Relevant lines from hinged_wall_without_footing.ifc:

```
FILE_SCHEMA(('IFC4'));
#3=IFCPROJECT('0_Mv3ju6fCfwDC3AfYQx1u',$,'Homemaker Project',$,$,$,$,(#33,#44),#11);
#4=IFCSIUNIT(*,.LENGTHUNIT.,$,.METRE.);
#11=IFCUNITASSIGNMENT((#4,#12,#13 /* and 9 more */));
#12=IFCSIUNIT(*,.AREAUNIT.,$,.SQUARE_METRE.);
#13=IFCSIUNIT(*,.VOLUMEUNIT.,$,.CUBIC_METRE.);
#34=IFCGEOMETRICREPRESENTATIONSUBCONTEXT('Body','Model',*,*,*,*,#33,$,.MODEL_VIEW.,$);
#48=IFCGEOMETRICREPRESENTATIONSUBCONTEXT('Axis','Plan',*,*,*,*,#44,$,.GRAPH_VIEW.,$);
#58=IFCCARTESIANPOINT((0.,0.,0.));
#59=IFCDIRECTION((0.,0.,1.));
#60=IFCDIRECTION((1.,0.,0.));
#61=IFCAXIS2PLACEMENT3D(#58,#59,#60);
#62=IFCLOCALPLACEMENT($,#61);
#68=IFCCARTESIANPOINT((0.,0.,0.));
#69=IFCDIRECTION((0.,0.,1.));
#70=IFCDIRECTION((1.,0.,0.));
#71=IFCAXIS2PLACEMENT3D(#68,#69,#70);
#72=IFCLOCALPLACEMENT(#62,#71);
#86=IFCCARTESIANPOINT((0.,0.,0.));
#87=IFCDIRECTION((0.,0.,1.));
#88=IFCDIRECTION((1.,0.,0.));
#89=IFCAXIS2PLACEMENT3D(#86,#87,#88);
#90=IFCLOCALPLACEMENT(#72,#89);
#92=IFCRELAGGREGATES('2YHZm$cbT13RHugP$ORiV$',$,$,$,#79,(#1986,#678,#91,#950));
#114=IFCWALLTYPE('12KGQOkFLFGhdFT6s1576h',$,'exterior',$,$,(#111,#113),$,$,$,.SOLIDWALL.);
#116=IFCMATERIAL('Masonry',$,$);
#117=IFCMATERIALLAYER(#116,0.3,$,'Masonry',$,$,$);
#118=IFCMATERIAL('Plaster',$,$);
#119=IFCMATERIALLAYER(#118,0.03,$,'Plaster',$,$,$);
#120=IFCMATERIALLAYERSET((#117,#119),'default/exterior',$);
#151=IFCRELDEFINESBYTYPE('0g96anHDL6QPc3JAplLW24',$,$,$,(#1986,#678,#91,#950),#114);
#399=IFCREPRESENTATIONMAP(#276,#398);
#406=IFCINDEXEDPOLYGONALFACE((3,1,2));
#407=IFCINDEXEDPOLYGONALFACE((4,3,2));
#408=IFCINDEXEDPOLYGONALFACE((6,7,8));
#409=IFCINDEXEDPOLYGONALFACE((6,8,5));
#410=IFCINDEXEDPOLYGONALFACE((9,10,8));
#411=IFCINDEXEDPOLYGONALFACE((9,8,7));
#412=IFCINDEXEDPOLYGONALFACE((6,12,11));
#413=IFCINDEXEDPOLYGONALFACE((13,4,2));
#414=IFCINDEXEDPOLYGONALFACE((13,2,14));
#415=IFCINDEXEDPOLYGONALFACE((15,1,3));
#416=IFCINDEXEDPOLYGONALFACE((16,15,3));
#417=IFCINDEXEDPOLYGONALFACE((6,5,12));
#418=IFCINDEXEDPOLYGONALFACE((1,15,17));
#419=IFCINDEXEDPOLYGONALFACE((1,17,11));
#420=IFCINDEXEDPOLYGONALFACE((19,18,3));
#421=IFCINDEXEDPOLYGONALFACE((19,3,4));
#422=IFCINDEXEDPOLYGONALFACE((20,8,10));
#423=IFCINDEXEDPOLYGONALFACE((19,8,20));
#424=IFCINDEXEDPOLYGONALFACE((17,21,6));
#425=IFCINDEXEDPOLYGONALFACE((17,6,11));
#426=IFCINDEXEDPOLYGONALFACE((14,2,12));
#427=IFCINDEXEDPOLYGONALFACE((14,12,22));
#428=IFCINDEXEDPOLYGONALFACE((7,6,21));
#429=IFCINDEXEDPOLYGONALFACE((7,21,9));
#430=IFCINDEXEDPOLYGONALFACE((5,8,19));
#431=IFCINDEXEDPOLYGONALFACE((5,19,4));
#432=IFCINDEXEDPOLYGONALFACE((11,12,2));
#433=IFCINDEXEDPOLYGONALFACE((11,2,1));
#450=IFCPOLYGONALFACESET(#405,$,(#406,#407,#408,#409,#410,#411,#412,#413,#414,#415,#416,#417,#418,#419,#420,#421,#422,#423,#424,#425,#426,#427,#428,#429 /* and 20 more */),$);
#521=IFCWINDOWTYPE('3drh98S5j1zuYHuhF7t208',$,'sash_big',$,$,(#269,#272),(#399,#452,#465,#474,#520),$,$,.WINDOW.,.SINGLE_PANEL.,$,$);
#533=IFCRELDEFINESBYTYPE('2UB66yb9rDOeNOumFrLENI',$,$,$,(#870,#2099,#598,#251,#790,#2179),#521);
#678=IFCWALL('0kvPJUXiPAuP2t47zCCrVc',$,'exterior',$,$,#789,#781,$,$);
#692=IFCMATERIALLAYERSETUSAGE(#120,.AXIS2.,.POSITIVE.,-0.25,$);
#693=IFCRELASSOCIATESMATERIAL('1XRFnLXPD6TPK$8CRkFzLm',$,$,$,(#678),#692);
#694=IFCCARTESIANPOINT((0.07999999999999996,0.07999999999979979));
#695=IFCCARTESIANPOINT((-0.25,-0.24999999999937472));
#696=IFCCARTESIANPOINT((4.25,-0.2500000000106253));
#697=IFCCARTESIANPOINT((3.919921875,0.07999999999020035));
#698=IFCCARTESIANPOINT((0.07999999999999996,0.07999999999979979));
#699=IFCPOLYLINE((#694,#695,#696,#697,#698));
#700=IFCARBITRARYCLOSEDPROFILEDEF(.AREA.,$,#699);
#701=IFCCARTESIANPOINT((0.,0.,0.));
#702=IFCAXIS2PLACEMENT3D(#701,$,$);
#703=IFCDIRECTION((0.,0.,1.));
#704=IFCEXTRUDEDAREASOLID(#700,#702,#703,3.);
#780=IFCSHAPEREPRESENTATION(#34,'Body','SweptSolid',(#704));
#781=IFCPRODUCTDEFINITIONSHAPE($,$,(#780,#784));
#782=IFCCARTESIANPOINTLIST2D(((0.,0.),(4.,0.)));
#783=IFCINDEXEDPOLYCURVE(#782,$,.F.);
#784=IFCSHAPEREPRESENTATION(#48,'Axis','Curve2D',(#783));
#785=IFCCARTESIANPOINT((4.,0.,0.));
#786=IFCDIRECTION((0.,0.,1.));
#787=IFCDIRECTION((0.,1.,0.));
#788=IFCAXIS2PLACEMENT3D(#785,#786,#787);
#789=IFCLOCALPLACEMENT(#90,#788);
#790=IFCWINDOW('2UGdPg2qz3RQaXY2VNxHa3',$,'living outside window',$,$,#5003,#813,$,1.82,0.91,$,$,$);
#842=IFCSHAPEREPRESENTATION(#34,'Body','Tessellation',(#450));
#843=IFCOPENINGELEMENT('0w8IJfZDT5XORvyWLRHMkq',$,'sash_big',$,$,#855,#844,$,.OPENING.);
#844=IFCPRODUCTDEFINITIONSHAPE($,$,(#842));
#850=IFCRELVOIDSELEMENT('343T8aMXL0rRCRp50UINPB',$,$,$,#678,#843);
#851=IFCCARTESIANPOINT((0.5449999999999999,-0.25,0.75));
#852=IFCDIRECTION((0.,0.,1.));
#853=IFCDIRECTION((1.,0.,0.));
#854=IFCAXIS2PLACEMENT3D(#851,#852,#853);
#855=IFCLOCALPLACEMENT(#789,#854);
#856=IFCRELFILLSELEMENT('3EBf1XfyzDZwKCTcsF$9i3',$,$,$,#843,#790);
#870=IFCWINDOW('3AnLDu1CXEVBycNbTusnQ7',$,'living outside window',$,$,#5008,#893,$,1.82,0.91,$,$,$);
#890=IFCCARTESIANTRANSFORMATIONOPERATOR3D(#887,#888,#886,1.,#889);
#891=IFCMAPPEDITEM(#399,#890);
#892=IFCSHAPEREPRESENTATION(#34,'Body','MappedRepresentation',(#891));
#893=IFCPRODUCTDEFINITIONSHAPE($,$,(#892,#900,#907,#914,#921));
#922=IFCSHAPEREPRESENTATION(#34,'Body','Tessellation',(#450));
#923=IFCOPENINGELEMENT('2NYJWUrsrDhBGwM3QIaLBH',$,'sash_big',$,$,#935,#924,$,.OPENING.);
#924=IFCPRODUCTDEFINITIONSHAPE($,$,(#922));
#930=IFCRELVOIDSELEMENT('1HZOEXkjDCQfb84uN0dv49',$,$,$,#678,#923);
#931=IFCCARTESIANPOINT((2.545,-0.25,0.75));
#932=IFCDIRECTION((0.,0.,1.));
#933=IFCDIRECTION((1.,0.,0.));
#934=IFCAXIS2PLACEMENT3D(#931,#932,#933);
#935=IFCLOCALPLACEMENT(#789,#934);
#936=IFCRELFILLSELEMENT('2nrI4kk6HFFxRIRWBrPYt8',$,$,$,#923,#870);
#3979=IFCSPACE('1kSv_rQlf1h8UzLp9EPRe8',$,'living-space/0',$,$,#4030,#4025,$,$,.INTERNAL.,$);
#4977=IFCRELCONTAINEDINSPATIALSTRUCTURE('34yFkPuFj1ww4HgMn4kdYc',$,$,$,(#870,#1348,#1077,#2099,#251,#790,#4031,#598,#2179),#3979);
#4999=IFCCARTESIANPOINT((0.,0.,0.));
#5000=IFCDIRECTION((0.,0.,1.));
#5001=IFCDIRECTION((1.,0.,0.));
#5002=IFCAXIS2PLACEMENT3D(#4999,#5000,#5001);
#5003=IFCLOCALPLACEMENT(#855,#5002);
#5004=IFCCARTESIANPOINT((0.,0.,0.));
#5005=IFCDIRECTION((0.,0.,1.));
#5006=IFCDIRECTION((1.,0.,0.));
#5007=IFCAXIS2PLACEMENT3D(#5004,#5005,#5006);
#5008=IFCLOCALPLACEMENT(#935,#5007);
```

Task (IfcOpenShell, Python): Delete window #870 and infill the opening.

```python
import ifcopenshell
import ifcopenshell.api.feature
import ifcopenshell.api.root
import ifcopenshell.geom
import ifcopenshell.util.shape

model = ifcopenshell.open("hinged_wall_without_footing.ifc")
settings = ifcopenshell.geom.settings()


def volume(element):
    """Net volume in cubic metres, openings subtracted."""
    shape = ifcopenshell.geom.create_shape(settings, element)
    return ifcopenshell.util.shape.get_volume(shape.geometry)


window = model.by_guid("3AnLDu1CXEVBycNbTusnQ7")
opening = window.FillsVoids[0].RelatingOpeningElement
wall = opening.VoidsElements[0].RelatingBuildingElement
before = volume(wall)

ifcopenshell.api.root.remove_product(model, product=window)
ifcopenshell.api.feature.remove_feature(model, feature=opening)

after = volume(wall)

print(f"wall volume {before:.3f} -> {after:.3f} m3")

model.write("hinged_wall_without_footing_v2.ifc")
```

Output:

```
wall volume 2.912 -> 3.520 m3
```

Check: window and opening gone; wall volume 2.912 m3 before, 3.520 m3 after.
